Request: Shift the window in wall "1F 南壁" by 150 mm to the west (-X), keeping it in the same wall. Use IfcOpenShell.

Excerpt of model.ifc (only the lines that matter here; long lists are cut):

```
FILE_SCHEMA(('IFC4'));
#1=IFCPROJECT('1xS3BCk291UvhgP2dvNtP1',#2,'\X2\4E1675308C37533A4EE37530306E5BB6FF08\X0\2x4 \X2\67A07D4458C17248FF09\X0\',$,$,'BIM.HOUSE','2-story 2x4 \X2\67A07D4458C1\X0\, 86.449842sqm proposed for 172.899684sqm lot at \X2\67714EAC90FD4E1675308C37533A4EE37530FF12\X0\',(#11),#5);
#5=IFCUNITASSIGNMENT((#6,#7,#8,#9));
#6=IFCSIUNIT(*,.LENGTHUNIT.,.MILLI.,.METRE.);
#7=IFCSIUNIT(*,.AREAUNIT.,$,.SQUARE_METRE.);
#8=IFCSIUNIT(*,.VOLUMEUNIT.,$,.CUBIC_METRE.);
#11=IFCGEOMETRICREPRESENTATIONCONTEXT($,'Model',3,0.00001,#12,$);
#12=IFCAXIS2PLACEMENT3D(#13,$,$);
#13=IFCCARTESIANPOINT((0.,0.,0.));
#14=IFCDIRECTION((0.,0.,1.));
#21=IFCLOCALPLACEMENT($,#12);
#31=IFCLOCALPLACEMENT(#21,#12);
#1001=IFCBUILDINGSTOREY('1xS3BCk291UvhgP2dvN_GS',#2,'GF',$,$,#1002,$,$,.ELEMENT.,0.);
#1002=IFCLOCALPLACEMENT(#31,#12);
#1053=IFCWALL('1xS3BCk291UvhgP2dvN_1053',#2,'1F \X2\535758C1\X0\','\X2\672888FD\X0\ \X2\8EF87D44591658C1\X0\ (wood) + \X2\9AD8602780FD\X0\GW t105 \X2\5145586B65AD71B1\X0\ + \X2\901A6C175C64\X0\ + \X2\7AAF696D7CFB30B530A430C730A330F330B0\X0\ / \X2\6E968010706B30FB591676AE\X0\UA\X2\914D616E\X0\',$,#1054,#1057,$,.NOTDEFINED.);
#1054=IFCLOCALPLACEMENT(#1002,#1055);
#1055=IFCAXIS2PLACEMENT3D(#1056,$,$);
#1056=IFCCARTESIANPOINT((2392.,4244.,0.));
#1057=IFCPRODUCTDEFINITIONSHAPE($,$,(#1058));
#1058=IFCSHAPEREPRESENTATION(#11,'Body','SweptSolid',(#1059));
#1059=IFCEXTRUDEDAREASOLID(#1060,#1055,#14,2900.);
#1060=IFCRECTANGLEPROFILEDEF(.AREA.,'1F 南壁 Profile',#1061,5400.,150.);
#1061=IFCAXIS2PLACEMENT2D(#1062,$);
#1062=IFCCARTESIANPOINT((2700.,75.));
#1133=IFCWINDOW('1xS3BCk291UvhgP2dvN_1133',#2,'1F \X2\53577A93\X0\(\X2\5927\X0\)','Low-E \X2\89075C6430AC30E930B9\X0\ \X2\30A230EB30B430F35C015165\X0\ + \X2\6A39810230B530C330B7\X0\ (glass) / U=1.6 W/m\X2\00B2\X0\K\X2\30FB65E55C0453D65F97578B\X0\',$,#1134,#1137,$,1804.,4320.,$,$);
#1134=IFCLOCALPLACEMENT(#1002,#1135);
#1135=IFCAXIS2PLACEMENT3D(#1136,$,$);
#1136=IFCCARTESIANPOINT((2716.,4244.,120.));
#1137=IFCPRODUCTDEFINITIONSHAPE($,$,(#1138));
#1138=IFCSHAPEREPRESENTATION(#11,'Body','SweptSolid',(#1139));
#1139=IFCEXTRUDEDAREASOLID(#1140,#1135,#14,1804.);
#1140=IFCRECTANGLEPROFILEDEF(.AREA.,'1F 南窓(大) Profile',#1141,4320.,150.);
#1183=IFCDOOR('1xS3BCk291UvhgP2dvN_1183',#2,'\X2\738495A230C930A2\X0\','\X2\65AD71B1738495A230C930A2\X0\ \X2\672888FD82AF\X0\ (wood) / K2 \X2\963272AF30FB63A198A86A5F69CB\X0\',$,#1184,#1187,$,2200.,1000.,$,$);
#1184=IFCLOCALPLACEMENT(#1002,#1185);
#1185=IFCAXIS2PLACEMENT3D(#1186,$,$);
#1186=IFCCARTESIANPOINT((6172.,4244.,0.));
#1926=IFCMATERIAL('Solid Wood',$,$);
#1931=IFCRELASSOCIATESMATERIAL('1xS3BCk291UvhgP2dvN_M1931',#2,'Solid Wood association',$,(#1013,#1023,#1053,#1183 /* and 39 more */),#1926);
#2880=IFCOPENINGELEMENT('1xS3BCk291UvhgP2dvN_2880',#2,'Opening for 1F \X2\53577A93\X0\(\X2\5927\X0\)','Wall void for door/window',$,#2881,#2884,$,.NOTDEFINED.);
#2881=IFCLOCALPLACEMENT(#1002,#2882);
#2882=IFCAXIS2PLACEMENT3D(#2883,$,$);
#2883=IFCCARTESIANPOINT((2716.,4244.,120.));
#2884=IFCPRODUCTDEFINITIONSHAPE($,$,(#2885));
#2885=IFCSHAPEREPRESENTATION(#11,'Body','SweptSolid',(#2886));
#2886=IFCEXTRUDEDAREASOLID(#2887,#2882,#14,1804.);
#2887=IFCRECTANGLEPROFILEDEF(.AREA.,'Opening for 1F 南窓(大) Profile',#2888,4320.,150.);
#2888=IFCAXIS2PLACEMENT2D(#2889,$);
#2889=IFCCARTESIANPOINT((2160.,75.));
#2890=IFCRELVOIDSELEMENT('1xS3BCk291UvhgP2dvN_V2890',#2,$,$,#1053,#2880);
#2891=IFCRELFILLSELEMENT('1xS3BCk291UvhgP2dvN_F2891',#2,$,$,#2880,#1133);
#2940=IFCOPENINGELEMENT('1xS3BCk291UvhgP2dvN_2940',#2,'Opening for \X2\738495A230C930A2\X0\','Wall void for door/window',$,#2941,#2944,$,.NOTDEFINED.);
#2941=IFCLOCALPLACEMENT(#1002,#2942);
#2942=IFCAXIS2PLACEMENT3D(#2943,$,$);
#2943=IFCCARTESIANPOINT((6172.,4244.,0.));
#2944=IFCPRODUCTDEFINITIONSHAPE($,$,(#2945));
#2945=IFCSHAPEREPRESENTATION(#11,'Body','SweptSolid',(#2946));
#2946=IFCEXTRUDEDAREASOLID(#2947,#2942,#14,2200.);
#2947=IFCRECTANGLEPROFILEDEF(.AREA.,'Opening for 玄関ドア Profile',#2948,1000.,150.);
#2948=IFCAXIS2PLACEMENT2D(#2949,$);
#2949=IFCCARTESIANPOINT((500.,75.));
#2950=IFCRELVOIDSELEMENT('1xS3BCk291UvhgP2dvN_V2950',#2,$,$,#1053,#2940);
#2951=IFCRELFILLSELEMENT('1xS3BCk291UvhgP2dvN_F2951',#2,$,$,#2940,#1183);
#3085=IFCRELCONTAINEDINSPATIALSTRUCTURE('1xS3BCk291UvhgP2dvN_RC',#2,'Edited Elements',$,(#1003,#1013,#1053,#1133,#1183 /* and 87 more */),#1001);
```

```python
import ifcopenshell
import ifcopenshell.api.geometry
import ifcopenshell.util.placement

model = ifcopenshell.open("model.ifc")

window = model.by_guid("1xS3BCk291UvhgP2dvN_1133")
opening = window.FillsVoids[0].RelatingOpeningElement
wall = opening.VoidsElements[0].RelatingBuildingElement

wall_matrix = ifcopenshell.util.placement.get_local_placement(wall.ObjectPlacement)
shift = wall_matrix[:3, 0] * -150.0
before = ifcopenshell.util.placement.get_local_placement(window.ObjectPlacement)[:3, 3].copy()

# The window is not placed relative to its opening, so move both.
for product in (opening, window):
    matrix = ifcopenshell.util.placement.get_local_placement(product.ObjectPlacement)
    matrix[:3, 3] += shift
    ifcopenshell.api.geometry.edit_object_placement(model, product=product, matrix=matrix, is_si=False)

after = ifcopenshell.util.placement.get_local_placement(window.ObjectPlacement)[:3, 3]
print("window moved by", (after - before).round(3) + 0.0)

model.write("model_rev.ifc")
```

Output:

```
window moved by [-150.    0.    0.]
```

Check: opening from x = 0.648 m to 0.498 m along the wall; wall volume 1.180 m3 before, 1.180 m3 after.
